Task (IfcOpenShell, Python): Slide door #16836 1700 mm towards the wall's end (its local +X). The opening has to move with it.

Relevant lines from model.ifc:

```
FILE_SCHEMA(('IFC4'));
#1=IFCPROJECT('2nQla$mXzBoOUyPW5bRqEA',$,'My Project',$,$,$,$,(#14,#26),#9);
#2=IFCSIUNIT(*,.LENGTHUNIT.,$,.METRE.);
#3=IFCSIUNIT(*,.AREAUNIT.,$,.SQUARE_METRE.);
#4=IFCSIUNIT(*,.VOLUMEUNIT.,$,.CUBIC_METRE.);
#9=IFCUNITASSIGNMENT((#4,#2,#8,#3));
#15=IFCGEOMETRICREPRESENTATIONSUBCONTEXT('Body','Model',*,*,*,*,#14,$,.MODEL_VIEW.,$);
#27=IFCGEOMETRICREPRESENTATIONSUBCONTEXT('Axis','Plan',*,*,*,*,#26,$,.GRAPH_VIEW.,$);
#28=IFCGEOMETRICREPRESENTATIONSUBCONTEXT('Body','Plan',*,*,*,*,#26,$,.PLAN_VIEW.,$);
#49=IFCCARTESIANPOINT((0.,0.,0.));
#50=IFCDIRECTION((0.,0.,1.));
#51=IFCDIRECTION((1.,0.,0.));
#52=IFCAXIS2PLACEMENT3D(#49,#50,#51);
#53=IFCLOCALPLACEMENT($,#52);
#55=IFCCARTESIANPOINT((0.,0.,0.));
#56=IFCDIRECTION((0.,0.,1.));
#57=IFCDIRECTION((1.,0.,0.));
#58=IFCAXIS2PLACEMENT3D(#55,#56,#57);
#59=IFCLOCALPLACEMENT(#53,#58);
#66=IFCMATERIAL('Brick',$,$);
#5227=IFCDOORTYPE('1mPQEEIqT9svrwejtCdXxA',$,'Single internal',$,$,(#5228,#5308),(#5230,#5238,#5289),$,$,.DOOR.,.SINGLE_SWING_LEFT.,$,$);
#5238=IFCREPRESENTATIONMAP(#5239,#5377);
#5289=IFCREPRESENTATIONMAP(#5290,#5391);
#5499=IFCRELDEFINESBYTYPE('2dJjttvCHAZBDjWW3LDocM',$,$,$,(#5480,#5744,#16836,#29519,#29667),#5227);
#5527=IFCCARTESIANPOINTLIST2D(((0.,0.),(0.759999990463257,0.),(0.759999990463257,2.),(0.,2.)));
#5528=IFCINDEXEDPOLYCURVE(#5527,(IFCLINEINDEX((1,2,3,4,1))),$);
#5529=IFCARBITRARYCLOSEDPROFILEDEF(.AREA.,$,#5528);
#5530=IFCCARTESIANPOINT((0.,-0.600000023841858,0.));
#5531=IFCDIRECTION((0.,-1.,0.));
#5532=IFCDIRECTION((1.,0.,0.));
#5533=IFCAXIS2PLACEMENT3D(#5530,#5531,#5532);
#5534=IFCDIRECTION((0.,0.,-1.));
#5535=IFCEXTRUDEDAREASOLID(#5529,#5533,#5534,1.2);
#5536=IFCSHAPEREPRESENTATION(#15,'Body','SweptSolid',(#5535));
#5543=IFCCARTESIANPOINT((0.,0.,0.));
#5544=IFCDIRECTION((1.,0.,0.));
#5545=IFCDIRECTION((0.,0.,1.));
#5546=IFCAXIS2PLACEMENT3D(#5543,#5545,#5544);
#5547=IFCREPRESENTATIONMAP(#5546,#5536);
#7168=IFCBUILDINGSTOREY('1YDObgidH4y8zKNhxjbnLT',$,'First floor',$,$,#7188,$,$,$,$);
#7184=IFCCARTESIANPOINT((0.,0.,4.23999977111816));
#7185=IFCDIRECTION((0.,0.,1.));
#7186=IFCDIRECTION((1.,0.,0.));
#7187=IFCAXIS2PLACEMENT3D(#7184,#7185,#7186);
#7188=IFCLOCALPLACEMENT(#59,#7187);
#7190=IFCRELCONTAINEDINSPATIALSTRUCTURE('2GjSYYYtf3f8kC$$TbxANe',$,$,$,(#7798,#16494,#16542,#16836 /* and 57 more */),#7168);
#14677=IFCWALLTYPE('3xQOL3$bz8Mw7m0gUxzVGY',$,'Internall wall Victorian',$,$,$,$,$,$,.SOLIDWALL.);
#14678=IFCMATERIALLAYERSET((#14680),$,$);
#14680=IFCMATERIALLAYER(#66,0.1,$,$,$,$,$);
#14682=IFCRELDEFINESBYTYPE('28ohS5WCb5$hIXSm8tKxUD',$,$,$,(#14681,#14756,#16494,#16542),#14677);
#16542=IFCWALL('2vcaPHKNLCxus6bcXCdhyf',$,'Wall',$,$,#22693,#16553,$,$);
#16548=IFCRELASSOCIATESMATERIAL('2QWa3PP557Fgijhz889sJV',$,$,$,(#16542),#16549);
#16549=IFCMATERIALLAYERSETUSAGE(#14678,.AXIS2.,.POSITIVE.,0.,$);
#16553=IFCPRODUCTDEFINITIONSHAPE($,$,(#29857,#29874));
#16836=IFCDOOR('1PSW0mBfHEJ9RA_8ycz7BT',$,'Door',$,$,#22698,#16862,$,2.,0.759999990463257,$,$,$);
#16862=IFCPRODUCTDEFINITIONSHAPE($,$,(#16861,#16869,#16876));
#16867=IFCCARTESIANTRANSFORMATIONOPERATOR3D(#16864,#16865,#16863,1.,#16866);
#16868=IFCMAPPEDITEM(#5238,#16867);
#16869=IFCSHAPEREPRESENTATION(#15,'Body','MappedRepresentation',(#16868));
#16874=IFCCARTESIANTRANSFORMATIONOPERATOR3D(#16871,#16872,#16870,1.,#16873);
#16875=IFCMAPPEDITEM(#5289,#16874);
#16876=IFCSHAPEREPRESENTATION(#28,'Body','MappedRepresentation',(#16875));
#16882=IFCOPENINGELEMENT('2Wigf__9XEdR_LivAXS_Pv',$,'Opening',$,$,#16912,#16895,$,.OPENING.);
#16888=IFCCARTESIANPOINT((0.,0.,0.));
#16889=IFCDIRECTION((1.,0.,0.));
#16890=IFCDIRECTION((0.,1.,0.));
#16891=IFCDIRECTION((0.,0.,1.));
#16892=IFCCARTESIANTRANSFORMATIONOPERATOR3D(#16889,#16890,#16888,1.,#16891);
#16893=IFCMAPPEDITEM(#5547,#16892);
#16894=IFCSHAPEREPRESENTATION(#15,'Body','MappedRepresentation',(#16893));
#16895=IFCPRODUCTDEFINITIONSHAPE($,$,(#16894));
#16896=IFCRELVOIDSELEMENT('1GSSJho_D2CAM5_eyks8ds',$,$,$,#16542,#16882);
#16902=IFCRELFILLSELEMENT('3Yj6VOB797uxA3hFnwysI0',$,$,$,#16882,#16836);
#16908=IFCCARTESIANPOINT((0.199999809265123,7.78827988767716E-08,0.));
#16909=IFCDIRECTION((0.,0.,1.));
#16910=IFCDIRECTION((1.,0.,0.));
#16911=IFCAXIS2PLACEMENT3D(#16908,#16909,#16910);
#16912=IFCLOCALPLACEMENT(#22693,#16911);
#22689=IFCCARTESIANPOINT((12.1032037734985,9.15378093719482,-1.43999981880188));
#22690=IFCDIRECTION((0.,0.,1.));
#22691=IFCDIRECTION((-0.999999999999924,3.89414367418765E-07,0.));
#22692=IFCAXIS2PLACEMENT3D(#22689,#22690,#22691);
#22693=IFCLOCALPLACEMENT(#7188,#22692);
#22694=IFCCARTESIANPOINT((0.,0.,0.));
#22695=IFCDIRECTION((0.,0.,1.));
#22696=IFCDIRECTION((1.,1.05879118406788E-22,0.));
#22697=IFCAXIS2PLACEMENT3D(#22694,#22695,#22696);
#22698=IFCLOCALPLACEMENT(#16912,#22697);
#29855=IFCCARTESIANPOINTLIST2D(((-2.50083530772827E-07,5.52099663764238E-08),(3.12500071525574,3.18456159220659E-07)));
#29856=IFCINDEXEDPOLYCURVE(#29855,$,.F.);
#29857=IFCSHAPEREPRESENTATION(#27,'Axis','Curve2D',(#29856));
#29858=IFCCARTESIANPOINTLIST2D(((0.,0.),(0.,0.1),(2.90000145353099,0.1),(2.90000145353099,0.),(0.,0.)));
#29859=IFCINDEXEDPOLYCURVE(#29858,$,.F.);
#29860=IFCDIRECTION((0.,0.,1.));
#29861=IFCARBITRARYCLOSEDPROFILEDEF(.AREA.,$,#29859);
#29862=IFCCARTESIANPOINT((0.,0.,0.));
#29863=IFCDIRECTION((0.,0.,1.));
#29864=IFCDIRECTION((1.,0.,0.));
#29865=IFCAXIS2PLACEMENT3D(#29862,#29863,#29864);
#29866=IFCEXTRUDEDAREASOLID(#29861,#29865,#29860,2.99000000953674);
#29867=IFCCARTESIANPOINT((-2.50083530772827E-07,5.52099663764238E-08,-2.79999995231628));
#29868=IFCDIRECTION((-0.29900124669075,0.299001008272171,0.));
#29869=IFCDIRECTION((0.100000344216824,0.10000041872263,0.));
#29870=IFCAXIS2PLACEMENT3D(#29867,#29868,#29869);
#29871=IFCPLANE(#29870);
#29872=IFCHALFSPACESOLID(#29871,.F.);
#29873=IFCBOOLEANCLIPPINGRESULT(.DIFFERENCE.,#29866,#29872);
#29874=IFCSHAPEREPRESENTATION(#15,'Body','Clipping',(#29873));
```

```python
import ifcopenshell
import ifcopenshell.api.geometry
import ifcopenshell.util.placement
import ifcopenshell.util.unit

model = ifcopenshell.open("model.ifc")
unit_scale = ifcopenshell.util.unit.calculate_unit_scale(model)

door = model.by_guid("1PSW0mBfHEJ9RA_8ycz7BT")
opening = door.FillsVoids[0].RelatingOpeningElement
wall = opening.VoidsElements[0].RelatingBuildingElement

wall_matrix = ifcopenshell.util.placement.get_local_placement(wall.ObjectPlacement)
shift = wall_matrix[:3, 0] * 1.7 / unit_scale
before = ifcopenshell.util.placement.get_local_placement(door.ObjectPlacement)[:3, 3].copy()

# The door is placed relative to its opening, so it follows when the opening moves.
matrix = ifcopenshell.util.placement.get_local_placement(opening.ObjectPlacement)
matrix[:3, 3] += shift
ifcopenshell.api.geometry.edit_object_placement(
    model, product=opening, matrix=matrix, is_si=False, should_transform_children=True
)

after = ifcopenshell.util.placement.get_local_placement(door.ObjectPlacement)[:3, 3]
print("door moved by", (after - before).round(3) + 0.0)

model.write("model-out.ifc")
```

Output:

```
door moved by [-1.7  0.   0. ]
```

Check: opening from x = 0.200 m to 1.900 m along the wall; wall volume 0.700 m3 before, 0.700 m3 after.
